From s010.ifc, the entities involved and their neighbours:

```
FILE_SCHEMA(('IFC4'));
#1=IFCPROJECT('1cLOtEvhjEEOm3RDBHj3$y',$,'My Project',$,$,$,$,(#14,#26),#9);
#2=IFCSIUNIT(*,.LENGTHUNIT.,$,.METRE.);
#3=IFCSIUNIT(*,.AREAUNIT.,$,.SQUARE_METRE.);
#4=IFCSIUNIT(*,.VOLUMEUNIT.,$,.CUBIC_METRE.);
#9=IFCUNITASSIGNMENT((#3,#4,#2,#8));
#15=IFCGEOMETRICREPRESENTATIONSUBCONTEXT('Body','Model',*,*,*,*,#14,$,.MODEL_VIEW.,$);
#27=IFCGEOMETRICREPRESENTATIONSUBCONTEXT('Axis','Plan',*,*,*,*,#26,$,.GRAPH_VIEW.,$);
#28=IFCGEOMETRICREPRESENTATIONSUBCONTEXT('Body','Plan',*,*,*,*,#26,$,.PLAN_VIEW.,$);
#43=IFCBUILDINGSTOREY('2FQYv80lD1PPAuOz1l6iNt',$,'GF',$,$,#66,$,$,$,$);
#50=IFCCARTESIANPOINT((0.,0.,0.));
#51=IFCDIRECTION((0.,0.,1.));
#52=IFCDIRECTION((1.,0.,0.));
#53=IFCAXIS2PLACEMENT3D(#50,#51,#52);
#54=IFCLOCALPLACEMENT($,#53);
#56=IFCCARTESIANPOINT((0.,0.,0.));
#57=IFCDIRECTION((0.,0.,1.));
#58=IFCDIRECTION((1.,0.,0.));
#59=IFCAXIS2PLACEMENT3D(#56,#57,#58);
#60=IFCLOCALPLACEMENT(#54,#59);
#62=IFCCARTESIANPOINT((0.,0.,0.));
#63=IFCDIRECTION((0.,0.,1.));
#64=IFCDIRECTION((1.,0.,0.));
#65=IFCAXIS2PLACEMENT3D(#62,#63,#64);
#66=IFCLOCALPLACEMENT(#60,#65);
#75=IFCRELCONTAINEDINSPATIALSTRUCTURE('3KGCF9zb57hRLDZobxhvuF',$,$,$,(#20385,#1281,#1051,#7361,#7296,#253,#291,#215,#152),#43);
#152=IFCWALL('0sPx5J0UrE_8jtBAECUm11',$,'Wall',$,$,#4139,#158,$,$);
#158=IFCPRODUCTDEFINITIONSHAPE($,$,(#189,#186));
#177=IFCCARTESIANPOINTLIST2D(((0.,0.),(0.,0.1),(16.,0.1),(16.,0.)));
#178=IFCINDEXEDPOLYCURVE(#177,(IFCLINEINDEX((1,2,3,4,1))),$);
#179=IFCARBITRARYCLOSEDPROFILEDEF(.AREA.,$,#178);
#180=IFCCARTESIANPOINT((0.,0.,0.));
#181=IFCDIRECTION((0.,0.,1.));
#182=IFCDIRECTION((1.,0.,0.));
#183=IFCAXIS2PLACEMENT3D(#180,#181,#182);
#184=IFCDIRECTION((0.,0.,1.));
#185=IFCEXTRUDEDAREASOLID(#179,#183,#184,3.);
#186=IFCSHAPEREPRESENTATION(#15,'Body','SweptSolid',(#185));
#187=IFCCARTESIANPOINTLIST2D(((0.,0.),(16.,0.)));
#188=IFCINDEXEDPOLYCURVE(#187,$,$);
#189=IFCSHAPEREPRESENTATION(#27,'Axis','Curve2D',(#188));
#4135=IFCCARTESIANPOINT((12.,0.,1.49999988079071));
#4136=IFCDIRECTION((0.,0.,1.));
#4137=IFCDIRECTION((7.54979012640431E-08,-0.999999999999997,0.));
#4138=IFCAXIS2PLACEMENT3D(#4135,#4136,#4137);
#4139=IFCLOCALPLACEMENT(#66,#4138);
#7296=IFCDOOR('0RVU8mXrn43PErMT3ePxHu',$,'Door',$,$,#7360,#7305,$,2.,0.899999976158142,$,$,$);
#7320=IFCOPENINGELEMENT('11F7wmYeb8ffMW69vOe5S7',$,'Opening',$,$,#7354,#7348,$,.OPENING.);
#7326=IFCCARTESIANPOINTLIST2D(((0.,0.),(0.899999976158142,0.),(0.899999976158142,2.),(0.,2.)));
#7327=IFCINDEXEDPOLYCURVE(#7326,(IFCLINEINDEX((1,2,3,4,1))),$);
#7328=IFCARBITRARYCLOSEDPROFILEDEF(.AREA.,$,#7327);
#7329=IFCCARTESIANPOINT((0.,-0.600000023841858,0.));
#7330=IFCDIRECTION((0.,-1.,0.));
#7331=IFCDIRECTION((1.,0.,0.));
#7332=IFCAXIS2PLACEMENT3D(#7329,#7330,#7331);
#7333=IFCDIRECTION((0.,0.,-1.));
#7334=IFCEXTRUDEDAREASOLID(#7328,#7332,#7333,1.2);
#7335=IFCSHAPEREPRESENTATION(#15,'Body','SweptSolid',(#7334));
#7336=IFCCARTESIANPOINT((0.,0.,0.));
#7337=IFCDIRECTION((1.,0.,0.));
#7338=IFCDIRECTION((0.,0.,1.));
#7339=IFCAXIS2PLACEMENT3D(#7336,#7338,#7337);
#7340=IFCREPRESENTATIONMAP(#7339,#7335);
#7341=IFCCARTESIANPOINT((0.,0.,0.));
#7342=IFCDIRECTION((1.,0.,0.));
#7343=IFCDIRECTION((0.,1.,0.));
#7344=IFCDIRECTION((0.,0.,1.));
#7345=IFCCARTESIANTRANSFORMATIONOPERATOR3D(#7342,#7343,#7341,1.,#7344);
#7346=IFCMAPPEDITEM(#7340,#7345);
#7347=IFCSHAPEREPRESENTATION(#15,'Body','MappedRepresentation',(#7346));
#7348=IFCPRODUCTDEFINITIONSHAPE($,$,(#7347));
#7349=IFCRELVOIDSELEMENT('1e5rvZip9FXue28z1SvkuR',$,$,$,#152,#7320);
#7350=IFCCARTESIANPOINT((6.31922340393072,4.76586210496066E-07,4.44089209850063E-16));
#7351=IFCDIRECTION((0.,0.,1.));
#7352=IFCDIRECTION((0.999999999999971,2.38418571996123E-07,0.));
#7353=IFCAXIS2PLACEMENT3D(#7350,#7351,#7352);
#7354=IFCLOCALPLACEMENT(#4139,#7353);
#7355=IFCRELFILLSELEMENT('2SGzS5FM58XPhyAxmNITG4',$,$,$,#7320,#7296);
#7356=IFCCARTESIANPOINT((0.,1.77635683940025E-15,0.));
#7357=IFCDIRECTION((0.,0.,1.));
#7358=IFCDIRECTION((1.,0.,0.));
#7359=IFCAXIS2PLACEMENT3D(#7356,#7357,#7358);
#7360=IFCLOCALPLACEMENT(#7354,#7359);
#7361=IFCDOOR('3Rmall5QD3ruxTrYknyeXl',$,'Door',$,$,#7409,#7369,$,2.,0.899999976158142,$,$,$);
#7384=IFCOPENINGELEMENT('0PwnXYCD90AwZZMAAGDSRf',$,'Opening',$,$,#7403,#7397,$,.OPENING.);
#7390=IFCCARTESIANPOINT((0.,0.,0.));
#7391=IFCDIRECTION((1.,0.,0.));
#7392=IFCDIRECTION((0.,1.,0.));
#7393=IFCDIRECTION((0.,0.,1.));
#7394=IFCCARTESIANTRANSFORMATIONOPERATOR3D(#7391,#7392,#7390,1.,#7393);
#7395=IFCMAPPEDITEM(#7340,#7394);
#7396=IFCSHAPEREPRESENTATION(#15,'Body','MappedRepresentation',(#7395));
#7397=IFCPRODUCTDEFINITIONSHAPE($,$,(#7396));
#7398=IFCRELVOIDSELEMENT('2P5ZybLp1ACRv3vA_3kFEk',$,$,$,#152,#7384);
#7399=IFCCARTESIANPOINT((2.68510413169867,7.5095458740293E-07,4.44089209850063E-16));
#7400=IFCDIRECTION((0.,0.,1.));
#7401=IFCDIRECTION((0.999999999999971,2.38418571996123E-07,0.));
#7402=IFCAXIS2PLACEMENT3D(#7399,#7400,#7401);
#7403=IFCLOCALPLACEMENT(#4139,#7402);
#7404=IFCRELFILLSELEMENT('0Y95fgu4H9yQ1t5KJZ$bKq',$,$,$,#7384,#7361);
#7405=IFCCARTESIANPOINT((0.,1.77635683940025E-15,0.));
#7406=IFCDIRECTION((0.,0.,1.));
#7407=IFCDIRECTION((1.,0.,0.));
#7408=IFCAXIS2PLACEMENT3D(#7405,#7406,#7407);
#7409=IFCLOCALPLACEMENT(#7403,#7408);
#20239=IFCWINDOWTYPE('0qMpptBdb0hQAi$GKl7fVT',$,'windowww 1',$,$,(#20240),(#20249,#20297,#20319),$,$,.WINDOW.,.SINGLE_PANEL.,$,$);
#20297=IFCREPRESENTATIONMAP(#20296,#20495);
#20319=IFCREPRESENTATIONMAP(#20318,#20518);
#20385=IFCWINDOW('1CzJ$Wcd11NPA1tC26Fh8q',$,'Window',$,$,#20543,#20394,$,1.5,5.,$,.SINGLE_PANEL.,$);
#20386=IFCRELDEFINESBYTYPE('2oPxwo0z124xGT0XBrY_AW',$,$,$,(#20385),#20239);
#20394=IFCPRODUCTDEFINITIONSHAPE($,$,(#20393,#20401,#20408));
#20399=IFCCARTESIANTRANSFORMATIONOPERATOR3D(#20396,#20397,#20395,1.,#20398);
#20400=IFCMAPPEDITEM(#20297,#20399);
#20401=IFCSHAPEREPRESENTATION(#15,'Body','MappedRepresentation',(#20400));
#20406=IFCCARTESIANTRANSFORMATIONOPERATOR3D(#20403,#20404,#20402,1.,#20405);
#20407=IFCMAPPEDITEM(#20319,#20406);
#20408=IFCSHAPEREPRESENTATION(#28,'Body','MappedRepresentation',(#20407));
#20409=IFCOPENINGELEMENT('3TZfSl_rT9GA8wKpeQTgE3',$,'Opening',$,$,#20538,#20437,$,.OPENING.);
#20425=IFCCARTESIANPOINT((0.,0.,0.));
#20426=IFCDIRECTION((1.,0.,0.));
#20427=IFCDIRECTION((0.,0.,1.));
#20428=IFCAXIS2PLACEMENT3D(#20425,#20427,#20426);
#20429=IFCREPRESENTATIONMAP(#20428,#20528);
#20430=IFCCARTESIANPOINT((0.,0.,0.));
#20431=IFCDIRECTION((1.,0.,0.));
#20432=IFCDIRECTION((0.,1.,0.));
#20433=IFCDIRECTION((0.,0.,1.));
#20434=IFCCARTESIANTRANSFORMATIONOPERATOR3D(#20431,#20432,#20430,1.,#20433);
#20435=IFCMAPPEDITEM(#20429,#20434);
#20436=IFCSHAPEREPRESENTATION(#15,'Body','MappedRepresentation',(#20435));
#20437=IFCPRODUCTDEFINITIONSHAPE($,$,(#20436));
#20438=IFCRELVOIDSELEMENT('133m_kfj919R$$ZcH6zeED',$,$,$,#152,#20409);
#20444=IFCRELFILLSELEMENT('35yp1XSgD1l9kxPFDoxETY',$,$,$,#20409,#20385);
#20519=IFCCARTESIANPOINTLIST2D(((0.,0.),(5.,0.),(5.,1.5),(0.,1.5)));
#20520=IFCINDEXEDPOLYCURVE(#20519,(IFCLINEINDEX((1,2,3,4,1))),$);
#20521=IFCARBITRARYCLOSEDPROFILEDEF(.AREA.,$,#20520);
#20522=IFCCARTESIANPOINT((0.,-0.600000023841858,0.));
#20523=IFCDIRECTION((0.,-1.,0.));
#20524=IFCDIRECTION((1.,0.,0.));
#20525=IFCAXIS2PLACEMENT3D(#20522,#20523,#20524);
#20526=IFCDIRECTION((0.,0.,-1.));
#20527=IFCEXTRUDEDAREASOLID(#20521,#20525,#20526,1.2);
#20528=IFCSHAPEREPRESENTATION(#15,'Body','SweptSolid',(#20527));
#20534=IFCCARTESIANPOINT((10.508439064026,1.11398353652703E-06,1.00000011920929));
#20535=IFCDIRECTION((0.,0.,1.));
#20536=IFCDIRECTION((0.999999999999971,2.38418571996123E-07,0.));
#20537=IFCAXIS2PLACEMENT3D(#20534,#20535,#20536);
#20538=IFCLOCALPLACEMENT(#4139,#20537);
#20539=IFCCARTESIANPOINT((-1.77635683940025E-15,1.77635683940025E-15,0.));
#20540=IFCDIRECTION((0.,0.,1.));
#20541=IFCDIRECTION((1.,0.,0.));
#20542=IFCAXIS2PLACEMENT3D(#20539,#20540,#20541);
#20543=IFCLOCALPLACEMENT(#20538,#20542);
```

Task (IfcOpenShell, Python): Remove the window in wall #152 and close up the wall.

```python
import ifcopenshell
import ifcopenshell.api.feature
import ifcopenshell.api.root
import ifcopenshell.geom
import ifcopenshell.util.shape

model = ifcopenshell.open("s010.ifc")
settings = ifcopenshell.geom.settings()


def volume(element):
    """Net volume in cubic metres, openings subtracted."""
    shape = ifcopenshell.geom.create_shape(settings, element)
    return ifcopenshell.util.shape.get_volume(shape.geometry)


window = model.by_guid("1CzJ$Wcd11NPA1tC26Fh8q")
opening = window.FillsVoids[0].RelatingOpeningElement
wall = opening.VoidsElements[0].RelatingBuildingElement
before = volume(wall)

ifcopenshell.api.root.remove_product(model, product=window)
ifcopenshell.api.feature.remove_feature(model, feature=opening)

after = volume(wall)

print(f"wall volume {before:.3f} -> {after:.3f} m3")

model.write("s010-out.ifc")
```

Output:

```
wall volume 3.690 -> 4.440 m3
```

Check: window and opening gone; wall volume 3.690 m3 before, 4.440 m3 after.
